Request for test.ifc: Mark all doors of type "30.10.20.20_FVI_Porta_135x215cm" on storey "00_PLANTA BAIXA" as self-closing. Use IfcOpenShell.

First a look at what the model holds.

```python
import ifcopenshell
import ifcopenshell.util.element

model = ifcopenshell.open("test.ifc")
print(model.schema)
storey = next(s for s in model.by_type("IfcBuildingStorey") if s.Name == "00_PLANTA BAIXA")
doors = [e for e in ifcopenshell.util.element.get_decomposition(storey) if e.is_a("IfcDoor")]
seen = {}
for e in doors:
    element_type = ifcopenshell.util.element.get_type(e)
    key = (element_type.Name if element_type != e and element_type else None, ifcopenshell.util.element.get_pset(e, "Pset_DoorCommon", "SelfClosing"))
    seen[key] = seen.get(key, 0) + 1
for (name, value), count in sorted(seen.items(), key=str):
    print(count, "x", name, "|", value)
```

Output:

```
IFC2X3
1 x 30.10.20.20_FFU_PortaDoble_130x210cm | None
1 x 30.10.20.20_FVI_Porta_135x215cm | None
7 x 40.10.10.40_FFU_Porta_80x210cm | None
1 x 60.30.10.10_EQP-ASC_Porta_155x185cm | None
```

```python
import ifcopenshell
import ifcopenshell.api.pset
import ifcopenshell.util.element

model = ifcopenshell.open("test.ifc")

storey = next(s for s in model.by_type("IfcBuildingStorey") if s.Name == "00_PLANTA BAIXA")
doors = [e for e in ifcopenshell.util.element.get_decomposition(storey) if e.is_a("IfcDoor")]

count = 0
for e in doors:
    element_type = ifcopenshell.util.element.get_type(e)
    if element_type in (None, e) or element_type.Name != "30.10.20.20_FVI_Porta_135x215cm":
        continue
    # add_pset returns the element's existing set when there is one.
    pset = ifcopenshell.api.pset.add_pset(model, product=e, name="Pset_DoorCommon")
    ifcopenshell.api.pset.edit_pset(model, pset=pset, properties={"SelfClosing": True})
    count += 1

print(count, "doors updated")

model.write("test_edited.ifc")
```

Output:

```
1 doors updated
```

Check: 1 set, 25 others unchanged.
